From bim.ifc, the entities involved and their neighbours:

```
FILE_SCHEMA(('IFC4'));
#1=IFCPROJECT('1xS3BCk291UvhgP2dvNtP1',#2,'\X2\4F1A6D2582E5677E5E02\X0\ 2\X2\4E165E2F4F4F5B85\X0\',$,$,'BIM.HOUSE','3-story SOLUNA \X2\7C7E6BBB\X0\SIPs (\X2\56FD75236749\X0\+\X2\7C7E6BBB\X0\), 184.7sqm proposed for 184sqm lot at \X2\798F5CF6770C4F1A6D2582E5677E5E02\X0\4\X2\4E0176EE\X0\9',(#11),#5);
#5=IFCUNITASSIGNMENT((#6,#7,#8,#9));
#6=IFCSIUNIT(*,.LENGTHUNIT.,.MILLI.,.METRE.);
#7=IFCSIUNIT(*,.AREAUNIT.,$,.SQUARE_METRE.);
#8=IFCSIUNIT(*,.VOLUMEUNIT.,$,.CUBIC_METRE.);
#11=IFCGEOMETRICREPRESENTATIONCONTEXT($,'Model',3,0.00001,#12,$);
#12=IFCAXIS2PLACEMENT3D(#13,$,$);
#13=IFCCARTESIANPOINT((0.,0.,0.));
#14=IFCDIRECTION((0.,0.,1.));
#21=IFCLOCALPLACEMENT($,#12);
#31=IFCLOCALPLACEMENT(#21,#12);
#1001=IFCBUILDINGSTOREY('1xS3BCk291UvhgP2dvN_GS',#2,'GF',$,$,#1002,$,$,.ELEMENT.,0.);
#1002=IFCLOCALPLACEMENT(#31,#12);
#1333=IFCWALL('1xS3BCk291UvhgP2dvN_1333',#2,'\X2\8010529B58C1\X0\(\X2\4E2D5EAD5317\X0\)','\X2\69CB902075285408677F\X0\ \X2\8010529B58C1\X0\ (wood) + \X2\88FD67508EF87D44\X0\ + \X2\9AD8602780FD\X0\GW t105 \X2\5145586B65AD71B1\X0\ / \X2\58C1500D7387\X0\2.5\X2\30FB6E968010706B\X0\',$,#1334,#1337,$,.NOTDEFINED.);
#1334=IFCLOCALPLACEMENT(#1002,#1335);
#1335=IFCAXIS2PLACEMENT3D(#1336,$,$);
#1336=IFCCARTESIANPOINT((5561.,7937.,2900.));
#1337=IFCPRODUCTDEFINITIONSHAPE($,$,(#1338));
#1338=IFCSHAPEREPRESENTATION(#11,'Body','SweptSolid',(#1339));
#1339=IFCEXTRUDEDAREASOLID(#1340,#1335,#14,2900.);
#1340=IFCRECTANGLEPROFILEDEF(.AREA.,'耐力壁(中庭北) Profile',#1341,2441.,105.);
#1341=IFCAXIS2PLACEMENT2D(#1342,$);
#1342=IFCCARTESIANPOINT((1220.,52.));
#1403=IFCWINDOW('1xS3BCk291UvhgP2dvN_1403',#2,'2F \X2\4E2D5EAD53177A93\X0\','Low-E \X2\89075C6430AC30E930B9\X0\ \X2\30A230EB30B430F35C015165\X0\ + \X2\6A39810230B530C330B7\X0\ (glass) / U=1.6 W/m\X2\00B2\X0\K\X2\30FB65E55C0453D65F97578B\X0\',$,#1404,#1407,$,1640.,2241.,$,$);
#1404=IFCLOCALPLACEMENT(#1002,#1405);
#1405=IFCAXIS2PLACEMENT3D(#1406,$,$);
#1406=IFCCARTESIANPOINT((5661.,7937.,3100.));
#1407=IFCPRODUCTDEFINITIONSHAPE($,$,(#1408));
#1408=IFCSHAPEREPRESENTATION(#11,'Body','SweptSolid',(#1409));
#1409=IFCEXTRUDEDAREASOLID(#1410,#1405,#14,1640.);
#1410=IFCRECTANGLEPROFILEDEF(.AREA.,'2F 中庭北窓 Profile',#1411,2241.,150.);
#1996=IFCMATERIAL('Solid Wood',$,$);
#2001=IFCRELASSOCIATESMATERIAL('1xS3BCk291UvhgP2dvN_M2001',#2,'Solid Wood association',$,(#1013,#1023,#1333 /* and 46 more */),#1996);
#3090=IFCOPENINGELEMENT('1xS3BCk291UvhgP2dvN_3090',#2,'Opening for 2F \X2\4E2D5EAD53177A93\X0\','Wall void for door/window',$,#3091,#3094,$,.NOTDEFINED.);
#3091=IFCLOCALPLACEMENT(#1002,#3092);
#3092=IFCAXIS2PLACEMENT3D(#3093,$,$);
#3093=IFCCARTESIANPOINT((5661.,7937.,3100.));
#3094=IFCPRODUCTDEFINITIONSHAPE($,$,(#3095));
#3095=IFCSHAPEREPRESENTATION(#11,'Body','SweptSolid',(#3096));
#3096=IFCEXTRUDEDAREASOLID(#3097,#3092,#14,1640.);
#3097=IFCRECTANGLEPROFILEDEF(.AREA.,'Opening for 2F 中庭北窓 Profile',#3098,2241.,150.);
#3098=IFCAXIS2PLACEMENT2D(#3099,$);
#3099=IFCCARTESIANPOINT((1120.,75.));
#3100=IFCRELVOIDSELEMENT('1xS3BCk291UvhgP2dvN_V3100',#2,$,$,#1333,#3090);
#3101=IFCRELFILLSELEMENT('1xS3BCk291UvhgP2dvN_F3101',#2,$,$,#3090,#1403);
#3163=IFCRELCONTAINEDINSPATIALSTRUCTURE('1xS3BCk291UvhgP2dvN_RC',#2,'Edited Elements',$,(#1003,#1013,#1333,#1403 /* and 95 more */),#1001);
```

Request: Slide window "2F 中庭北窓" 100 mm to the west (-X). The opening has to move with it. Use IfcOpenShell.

```python
import ifcopenshell
import ifcopenshell.api.geometry
import ifcopenshell.util.placement
import ifcopenshell.util.unit

model = ifcopenshell.open("bim.ifc")
unit_scale = ifcopenshell.util.unit.calculate_unit_scale(model)

window = model.by_guid("1xS3BCk291UvhgP2dvN_1403")
opening = window.FillsVoids[0].RelatingOpeningElement
wall = opening.VoidsElements[0].RelatingBuildingElement

wall_matrix = ifcopenshell.util.placement.get_local_placement(wall.ObjectPlacement)
shift = wall_matrix[:3, 0] * -0.1 / unit_scale
before = ifcopenshell.util.placement.get_local_placement(window.ObjectPlacement)[:3, 3].copy()

# The window is not placed relative to its opening, so move both.
for product in (opening, window):
    matrix = ifcopenshell.util.placement.get_local_placement(product.ObjectPlacement)
    matrix[:3, 3] += shift
    ifcopenshell.api.geometry.edit_object_placement(model, product=product, matrix=matrix, is_si=False)

after = ifcopenshell.util.placement.get_local_placement(window.ObjectPlacement)[:3, 3]
print("window moved by", (after - before).round(3) + 0.0)

model.write("bim_edited.ifc")
```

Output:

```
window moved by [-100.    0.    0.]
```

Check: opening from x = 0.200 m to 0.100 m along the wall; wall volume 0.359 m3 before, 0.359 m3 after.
